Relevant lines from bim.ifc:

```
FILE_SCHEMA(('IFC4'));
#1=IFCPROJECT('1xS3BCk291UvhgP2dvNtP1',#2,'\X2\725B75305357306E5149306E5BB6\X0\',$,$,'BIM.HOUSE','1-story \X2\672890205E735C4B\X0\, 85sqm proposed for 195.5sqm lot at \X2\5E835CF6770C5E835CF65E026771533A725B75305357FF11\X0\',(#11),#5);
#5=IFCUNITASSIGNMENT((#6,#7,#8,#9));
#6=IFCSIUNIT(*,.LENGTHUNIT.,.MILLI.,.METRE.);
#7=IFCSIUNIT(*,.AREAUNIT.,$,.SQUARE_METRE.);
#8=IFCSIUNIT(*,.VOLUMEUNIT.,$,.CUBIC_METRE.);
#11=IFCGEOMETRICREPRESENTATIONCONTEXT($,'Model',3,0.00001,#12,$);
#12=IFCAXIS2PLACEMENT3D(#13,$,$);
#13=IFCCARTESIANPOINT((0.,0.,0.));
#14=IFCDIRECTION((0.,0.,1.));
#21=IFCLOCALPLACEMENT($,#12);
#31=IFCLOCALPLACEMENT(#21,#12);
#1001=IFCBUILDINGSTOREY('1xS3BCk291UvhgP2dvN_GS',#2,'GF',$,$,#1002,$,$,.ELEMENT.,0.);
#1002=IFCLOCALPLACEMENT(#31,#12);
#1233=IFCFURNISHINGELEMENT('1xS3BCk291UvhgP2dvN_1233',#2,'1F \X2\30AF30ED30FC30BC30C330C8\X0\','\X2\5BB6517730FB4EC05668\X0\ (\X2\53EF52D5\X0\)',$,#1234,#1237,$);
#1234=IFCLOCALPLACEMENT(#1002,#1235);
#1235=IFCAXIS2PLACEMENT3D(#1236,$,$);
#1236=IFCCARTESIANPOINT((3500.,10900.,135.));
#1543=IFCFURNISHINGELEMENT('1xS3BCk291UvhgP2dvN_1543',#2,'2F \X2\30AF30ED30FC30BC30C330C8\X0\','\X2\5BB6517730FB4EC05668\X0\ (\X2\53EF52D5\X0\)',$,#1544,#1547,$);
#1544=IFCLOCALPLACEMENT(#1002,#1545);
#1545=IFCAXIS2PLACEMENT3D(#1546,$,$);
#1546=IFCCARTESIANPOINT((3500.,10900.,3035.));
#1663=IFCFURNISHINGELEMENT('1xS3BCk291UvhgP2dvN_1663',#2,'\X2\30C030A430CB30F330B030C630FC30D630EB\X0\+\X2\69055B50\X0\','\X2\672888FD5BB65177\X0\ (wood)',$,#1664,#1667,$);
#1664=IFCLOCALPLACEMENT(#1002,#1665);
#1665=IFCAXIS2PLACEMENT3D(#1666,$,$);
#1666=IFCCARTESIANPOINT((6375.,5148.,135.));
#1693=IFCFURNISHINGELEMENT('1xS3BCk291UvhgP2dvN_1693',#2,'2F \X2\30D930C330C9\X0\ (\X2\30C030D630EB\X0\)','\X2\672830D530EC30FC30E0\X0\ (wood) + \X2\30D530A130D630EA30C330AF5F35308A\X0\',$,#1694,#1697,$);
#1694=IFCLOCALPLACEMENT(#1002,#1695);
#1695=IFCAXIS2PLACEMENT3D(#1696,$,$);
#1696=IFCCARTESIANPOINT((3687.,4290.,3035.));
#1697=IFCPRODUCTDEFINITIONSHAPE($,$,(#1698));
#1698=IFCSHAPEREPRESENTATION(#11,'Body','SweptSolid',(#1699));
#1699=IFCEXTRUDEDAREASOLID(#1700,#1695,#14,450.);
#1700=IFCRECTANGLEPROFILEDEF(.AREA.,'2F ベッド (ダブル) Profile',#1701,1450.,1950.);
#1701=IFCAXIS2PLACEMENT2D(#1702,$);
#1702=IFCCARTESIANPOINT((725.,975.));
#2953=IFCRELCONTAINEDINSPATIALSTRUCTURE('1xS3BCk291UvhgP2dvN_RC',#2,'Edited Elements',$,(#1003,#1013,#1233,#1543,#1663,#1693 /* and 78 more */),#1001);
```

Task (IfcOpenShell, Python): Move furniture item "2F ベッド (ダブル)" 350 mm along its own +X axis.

```python
import ifcopenshell
import ifcopenshell.api.geometry
import ifcopenshell.util.placement

model = ifcopenshell.open("bim.ifc")

item = model.by_guid("1xS3BCk291UvhgP2dvN_1693")
matrix = ifcopenshell.util.placement.get_local_placement(item.ObjectPlacement)
matrix[:3, 3] += matrix[:3, 0] * 350.0
ifcopenshell.api.geometry.edit_object_placement(model, product=item, matrix=matrix, is_si=False)

print(ifcopenshell.util.placement.get_local_placement(item.ObjectPlacement).round(3) + 0.0)

model.write("bim_rev.ifc")
```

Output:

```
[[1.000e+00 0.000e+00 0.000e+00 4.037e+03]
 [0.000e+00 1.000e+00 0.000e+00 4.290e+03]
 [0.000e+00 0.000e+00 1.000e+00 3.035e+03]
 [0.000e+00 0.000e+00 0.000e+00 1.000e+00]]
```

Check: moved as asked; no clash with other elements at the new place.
